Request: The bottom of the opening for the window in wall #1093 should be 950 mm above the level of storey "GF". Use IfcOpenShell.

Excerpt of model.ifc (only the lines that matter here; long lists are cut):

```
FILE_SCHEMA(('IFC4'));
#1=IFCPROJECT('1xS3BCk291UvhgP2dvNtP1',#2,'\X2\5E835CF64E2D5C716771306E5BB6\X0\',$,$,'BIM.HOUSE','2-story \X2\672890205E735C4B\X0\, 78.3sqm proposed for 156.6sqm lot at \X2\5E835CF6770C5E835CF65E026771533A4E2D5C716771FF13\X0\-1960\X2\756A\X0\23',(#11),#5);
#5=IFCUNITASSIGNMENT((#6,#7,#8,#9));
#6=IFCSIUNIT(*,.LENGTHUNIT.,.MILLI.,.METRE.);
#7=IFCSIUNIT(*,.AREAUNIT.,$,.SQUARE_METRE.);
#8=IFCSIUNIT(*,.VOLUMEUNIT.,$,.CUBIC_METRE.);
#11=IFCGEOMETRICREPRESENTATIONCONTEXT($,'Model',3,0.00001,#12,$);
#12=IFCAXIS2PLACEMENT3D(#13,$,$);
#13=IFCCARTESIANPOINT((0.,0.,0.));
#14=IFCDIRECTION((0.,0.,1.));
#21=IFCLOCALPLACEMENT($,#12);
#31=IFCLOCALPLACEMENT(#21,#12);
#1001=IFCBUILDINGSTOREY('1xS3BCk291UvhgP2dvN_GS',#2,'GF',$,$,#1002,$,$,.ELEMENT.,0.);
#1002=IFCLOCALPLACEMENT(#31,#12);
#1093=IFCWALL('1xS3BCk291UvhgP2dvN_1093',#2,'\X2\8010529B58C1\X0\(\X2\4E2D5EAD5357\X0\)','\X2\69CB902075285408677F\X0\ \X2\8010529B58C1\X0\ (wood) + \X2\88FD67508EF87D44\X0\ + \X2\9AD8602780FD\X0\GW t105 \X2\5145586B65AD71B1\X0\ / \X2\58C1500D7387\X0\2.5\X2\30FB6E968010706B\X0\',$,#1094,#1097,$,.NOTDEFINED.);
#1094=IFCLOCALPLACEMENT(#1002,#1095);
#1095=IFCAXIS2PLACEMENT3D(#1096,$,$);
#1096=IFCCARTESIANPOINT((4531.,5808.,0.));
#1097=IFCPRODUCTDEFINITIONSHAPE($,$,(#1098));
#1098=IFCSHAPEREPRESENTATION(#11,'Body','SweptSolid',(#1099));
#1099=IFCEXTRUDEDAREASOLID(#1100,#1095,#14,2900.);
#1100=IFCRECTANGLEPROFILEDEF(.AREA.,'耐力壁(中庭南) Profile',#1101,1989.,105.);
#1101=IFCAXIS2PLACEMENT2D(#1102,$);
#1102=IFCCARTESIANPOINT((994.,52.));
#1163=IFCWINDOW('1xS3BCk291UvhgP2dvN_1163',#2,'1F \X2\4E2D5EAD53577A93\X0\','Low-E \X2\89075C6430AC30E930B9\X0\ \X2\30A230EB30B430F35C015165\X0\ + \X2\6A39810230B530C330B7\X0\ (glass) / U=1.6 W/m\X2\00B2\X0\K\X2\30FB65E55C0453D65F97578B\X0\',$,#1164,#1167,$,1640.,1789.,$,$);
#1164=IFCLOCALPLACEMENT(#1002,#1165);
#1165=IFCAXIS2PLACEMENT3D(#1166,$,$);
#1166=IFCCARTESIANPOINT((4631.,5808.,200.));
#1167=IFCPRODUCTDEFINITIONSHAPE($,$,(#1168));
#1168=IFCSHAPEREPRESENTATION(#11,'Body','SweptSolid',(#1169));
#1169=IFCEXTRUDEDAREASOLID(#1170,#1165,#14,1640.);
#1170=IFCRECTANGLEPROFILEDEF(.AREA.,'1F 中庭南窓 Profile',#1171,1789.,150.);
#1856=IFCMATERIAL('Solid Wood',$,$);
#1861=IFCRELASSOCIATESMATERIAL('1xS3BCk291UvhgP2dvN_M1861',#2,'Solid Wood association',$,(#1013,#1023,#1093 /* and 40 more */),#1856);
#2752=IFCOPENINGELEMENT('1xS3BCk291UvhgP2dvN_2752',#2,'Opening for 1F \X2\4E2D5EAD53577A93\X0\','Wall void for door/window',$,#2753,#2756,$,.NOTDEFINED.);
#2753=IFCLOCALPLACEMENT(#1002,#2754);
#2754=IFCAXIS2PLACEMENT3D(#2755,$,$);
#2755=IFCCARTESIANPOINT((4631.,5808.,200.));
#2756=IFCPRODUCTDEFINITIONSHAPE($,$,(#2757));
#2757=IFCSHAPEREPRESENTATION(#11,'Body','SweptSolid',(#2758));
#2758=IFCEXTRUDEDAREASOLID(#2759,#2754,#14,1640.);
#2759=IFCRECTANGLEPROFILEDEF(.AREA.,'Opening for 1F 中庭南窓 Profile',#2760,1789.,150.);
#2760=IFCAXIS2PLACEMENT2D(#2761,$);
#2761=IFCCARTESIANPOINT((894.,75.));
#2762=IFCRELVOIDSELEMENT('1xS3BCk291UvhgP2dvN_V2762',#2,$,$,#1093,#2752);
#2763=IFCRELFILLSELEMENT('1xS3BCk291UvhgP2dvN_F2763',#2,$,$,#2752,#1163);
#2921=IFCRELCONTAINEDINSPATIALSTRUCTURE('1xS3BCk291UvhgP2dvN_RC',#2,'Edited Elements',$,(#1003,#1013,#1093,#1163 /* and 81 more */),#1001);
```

```python
import numpy as np
import ifcopenshell
import ifcopenshell.api.geometry
import ifcopenshell.geom
import ifcopenshell.util.element
import ifcopenshell.util.placement
import ifcopenshell.util.shape
import ifcopenshell.util.unit

model = ifcopenshell.open("model.ifc")
unit_scale = ifcopenshell.util.unit.calculate_unit_scale(model)

window = model.by_guid("1xS3BCk291UvhgP2dvN_1163")
opening = window.FillsVoids[0].RelatingOpeningElement
storey = ifcopenshell.util.element.get_container(window, ifc_class="IfcBuildingStorey")
level = ifcopenshell.util.placement.get_local_placement(storey.ObjectPlacement)[2, 3]

# The opening's origin need not be at the sill, so measure its lowest point.
shape = ifcopenshell.geom.create_shape(ifcopenshell.geom.settings(), opening)
bottom = ifcopenshell.util.shape.get_shape_bottom_elevation(shape, shape.geometry) / unit_scale
dz = level + 0.95 / unit_scale - bottom

shift = np.array([0.0, 0.0, dz])
# The window is not placed relative to its opening, so move both.
for product in (opening, window):
    matrix = ifcopenshell.util.placement.get_local_placement(product.ObjectPlacement)
    matrix[:3, 3] += shift
    ifcopenshell.api.geometry.edit_object_placement(model, product=product, matrix=matrix, is_si=False)

print(f"moved by {dz * unit_scale:+.3f} m")

model.write("model_rev.ifc")
```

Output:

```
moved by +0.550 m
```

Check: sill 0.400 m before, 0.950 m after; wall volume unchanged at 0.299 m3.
